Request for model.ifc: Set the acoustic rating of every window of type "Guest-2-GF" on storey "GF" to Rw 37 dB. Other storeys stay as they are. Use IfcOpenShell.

First a look at what the model holds.

```python
import ifcopenshell
import ifcopenshell.util.element

model = ifcopenshell.open("model.ifc")
print(model.schema)
storey = next(s for s in model.by_type("IfcBuildingStorey") if s.Name == "GF")
windows = [e for e in ifcopenshell.util.element.get_decomposition(storey) if e.is_a("IfcWindow")]
seen = {}
for e in windows:
    element_type = ifcopenshell.util.element.get_type(e)
    key = (element_type.Name if element_type != e and element_type else None, ifcopenshell.util.element.get_pset(e, "Pset_WindowCommon", "AcousticRating"))
    seen[key] = seen.get(key, 0) + 1
for (name, value), count in sorted(seen.items(), key=str):
    print(count, "x", name, "|", value)
```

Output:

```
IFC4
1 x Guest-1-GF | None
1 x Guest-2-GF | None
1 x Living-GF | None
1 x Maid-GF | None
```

```python
import ifcopenshell
import ifcopenshell.api.pset
import ifcopenshell.util.element

model = ifcopenshell.open("model.ifc")

storey = next(s for s in model.by_type("IfcBuildingStorey") if s.Name == "GF")
windows = [e for e in ifcopenshell.util.element.get_decomposition(storey) if e.is_a("IfcWindow")]

count = 0
for e in windows:
    element_type = ifcopenshell.util.element.get_type(e)
    if element_type in (None, e) or element_type.Name != "Guest-2-GF":
        continue
    # add_pset returns the element's existing set when there is one.
    pset = ifcopenshell.api.pset.add_pset(model, product=e, name="Pset_WindowCommon")
    ifcopenshell.api.pset.edit_pset(model, pset=pset, properties={"AcousticRating": "Rw 37 dB"})
    count += 1

print(count, "windows updated")

model.write("model_updated.ifc")
```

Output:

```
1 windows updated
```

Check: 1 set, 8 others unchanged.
